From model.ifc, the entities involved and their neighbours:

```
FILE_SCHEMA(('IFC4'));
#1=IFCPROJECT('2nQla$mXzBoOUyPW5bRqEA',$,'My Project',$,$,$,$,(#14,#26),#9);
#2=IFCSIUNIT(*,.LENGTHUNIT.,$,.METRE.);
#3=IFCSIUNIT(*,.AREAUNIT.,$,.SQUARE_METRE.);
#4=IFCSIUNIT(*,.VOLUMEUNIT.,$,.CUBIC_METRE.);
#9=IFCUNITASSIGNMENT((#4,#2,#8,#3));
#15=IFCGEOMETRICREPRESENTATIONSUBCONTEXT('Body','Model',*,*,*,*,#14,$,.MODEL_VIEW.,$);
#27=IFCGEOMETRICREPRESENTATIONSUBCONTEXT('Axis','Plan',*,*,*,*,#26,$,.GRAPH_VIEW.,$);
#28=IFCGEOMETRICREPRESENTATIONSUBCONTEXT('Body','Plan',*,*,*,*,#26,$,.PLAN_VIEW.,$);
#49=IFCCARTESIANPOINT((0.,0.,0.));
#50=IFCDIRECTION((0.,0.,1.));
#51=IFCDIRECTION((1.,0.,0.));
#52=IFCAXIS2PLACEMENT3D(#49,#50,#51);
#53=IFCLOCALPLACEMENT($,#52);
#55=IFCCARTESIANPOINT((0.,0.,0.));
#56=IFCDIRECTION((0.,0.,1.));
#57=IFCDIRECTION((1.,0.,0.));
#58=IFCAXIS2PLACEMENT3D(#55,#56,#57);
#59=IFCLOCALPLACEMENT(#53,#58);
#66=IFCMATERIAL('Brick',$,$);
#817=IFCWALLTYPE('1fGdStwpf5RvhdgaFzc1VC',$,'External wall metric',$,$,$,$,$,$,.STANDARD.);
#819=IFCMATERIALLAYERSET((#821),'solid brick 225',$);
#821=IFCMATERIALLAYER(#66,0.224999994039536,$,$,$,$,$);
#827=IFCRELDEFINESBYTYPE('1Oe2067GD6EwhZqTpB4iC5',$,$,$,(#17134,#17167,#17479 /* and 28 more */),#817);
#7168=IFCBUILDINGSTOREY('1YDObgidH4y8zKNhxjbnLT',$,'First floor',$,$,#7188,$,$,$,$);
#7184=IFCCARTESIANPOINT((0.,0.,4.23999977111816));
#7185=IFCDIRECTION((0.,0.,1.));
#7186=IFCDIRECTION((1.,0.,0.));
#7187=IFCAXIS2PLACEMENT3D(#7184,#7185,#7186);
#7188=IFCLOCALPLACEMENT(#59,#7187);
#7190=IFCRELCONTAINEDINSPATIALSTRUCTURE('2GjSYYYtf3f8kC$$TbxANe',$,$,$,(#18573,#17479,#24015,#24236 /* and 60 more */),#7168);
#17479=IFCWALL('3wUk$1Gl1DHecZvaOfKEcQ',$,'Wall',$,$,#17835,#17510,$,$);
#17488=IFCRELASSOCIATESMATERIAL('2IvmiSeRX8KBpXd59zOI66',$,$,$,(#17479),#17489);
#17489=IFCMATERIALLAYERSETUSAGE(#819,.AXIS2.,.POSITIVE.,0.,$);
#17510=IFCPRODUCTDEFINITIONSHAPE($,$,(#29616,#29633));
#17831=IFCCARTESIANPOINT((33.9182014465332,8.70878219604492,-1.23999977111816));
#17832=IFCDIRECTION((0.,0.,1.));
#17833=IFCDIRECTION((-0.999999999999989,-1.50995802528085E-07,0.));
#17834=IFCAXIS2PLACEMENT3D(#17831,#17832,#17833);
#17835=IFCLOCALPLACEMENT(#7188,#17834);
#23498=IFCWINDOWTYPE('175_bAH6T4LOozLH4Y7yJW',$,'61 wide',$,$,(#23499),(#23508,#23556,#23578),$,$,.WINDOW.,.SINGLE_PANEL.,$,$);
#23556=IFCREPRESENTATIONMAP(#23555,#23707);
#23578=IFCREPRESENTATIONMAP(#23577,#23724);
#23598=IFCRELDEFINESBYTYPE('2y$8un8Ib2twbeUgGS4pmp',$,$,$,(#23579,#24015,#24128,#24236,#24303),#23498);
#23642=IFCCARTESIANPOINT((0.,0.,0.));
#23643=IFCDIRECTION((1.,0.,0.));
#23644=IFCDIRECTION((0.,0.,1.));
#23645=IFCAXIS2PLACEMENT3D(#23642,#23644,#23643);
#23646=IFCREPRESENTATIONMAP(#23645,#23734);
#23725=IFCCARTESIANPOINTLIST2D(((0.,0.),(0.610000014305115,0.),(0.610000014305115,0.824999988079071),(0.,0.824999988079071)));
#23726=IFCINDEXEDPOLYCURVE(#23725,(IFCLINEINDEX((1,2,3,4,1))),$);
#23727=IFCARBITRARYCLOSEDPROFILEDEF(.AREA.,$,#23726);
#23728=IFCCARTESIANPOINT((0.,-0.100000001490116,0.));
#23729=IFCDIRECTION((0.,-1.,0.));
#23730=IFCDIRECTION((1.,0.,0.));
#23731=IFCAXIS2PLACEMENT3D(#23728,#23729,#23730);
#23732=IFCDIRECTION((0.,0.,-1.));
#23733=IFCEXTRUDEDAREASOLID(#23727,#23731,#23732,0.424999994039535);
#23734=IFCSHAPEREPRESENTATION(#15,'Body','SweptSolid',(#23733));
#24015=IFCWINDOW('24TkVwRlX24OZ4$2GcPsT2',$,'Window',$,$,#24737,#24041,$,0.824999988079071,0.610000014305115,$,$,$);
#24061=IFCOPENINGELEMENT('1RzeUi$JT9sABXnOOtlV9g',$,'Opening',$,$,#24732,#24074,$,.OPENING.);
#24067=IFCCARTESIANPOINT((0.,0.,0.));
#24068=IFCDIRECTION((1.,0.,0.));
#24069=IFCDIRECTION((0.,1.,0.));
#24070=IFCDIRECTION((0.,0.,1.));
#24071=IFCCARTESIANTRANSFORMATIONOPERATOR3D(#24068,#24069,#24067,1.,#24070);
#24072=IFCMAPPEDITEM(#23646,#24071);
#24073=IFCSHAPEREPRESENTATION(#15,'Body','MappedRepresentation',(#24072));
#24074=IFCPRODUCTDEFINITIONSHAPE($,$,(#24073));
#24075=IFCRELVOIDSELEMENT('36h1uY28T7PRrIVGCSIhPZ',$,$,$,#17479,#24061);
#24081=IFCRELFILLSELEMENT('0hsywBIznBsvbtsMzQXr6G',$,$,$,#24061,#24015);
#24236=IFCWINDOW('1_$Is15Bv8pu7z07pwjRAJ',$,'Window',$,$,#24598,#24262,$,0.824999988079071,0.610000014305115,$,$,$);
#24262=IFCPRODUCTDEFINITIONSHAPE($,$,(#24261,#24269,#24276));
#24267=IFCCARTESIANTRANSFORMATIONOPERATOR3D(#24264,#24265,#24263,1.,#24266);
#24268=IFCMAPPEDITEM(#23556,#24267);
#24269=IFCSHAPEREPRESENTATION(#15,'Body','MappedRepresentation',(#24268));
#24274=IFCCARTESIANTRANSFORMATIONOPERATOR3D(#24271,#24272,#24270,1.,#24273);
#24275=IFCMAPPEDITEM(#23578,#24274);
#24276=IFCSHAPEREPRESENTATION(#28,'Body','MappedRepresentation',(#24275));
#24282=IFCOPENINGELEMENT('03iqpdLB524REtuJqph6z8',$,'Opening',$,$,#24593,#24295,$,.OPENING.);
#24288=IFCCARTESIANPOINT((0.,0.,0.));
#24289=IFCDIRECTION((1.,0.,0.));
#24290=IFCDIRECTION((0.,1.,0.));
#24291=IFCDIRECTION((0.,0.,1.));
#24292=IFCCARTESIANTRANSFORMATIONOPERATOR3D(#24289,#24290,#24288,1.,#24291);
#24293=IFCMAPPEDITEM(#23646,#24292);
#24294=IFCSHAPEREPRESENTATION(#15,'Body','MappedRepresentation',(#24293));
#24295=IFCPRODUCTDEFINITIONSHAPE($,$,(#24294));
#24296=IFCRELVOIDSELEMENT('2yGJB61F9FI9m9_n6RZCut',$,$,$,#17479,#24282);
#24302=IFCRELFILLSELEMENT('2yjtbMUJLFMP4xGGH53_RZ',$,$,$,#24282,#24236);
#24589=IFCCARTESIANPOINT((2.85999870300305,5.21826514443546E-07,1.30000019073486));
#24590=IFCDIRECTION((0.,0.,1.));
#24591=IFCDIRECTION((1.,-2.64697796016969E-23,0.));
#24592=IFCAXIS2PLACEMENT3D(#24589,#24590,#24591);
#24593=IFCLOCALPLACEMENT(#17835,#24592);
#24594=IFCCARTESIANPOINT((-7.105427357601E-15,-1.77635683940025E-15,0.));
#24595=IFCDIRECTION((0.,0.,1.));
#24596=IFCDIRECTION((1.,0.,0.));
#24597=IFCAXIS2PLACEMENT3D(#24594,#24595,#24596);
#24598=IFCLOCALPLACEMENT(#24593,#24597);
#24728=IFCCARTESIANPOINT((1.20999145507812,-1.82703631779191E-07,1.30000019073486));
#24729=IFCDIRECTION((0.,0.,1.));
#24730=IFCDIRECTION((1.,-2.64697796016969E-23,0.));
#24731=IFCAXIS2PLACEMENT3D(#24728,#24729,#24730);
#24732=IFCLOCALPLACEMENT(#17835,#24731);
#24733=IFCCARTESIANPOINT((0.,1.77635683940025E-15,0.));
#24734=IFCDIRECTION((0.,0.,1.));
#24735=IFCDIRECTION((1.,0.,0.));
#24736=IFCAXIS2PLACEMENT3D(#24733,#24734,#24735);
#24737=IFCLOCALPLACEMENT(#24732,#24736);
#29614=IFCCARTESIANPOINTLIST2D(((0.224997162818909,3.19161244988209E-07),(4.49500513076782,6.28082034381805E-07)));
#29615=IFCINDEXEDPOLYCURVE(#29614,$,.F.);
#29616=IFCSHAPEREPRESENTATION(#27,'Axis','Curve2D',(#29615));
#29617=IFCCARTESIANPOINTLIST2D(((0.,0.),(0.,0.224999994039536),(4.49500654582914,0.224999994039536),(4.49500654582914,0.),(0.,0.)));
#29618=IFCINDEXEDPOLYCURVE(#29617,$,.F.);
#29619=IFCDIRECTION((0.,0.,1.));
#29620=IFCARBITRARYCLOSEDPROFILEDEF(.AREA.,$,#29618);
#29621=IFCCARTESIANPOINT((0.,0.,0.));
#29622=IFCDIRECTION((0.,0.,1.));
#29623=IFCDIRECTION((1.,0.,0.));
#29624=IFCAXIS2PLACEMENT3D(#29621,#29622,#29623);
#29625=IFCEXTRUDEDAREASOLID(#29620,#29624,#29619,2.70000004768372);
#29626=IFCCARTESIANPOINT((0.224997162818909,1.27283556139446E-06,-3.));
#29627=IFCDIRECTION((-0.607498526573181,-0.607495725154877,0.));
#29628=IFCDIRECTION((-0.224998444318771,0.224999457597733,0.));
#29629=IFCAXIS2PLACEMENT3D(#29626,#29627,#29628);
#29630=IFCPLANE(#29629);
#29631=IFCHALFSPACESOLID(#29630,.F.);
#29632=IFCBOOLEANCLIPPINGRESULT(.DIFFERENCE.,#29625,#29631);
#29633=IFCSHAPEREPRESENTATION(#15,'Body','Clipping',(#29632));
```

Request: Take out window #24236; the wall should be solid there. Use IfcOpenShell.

```python
import ifcopenshell
import ifcopenshell.api.feature
import ifcopenshell.api.root
import ifcopenshell.geom
import ifcopenshell.util.shape

model = ifcopenshell.open("model.ifc")
settings = ifcopenshell.geom.settings()


def volume(element):
    """Net volume in cubic metres, openings subtracted."""
    shape = ifcopenshell.geom.create_shape(settings, element)
    return ifcopenshell.util.shape.get_volume(shape.geometry)


window = model.by_guid("1_$Is15Bv8pu7z07pwjRAJ")
opening = window.FillsVoids[0].RelatingOpeningElement
wall = opening.VoidsElements[0].RelatingBuildingElement
before = volume(wall)

ifcopenshell.api.root.remove_product(model, product=window)
ifcopenshell.api.feature.remove_feature(model, feature=opening)

after = volume(wall)

print(f"wall volume {before:.3f} -> {after:.3f} m3")

model.write("model_rev.ifc")
```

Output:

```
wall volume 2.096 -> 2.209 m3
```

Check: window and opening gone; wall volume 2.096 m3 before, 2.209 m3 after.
